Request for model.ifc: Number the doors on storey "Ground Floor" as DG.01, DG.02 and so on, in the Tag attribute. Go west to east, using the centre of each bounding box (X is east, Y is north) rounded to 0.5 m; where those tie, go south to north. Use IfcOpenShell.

First a look at what the model holds.

```python
import ifcopenshell
import ifcopenshell.util.element
import ifcopenshell.util.placement

model = ifcopenshell.open("model.ifc")
print(model.schema)
storey = next(s for s in model.by_type("IfcBuildingStorey") if s.Name == "Ground Floor")
doors = [e for e in ifcopenshell.util.element.get_decomposition(storey) if e.is_a("IfcDoor")]
for e in sorted(doors, key=lambda e: e.id()):
    origin = ifcopenshell.util.placement.get_local_placement(e.ObjectPlacement)[:3, 3]
    print(e.id(), e.Tag, e.Name, origin.round(2) + 0.0, sep=" | ")
```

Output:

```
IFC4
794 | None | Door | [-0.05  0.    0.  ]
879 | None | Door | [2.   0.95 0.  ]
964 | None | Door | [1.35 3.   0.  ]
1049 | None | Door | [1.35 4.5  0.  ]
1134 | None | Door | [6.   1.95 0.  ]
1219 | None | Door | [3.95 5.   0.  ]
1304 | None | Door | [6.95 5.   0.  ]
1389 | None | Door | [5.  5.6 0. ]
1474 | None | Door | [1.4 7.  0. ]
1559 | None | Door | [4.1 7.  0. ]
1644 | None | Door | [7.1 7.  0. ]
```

```python
import ifcopenshell
import ifcopenshell.geom
import ifcopenshell.util.element
import ifcopenshell.util.shape

model = ifcopenshell.open("model.ifc")
settings = ifcopenshell.geom.settings()
settings.set("use-world-coords", True)


def centre(element):
    shape = ifcopenshell.geom.create_shape(settings, element)
    return ifcopenshell.util.shape.get_bbox_centroid(shape.geometry)


storey = next(s for s in model.by_type("IfcBuildingStorey") if s.Name == "Ground Floor")
doors = [e for e in ifcopenshell.util.element.get_decomposition(storey) if e.is_a("IfcDoor")]

# Insertion points can sit at a corner or the storey origin, so sort by the geometry (in metres).
centres = {e: centre(e) for e in doors}
doors.sort(key=lambda e: (round(centres[e][0] / 0.5), centres[e][1]))

for i, e in enumerate(doors, start=1):
    number = f"DG.{i:02d}"
    e.Tag = number
    print(e.id(), number)

model.write("model_rev.ifc")
```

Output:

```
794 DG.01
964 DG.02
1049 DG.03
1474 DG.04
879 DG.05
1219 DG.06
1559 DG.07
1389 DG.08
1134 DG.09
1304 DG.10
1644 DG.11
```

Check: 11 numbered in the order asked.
